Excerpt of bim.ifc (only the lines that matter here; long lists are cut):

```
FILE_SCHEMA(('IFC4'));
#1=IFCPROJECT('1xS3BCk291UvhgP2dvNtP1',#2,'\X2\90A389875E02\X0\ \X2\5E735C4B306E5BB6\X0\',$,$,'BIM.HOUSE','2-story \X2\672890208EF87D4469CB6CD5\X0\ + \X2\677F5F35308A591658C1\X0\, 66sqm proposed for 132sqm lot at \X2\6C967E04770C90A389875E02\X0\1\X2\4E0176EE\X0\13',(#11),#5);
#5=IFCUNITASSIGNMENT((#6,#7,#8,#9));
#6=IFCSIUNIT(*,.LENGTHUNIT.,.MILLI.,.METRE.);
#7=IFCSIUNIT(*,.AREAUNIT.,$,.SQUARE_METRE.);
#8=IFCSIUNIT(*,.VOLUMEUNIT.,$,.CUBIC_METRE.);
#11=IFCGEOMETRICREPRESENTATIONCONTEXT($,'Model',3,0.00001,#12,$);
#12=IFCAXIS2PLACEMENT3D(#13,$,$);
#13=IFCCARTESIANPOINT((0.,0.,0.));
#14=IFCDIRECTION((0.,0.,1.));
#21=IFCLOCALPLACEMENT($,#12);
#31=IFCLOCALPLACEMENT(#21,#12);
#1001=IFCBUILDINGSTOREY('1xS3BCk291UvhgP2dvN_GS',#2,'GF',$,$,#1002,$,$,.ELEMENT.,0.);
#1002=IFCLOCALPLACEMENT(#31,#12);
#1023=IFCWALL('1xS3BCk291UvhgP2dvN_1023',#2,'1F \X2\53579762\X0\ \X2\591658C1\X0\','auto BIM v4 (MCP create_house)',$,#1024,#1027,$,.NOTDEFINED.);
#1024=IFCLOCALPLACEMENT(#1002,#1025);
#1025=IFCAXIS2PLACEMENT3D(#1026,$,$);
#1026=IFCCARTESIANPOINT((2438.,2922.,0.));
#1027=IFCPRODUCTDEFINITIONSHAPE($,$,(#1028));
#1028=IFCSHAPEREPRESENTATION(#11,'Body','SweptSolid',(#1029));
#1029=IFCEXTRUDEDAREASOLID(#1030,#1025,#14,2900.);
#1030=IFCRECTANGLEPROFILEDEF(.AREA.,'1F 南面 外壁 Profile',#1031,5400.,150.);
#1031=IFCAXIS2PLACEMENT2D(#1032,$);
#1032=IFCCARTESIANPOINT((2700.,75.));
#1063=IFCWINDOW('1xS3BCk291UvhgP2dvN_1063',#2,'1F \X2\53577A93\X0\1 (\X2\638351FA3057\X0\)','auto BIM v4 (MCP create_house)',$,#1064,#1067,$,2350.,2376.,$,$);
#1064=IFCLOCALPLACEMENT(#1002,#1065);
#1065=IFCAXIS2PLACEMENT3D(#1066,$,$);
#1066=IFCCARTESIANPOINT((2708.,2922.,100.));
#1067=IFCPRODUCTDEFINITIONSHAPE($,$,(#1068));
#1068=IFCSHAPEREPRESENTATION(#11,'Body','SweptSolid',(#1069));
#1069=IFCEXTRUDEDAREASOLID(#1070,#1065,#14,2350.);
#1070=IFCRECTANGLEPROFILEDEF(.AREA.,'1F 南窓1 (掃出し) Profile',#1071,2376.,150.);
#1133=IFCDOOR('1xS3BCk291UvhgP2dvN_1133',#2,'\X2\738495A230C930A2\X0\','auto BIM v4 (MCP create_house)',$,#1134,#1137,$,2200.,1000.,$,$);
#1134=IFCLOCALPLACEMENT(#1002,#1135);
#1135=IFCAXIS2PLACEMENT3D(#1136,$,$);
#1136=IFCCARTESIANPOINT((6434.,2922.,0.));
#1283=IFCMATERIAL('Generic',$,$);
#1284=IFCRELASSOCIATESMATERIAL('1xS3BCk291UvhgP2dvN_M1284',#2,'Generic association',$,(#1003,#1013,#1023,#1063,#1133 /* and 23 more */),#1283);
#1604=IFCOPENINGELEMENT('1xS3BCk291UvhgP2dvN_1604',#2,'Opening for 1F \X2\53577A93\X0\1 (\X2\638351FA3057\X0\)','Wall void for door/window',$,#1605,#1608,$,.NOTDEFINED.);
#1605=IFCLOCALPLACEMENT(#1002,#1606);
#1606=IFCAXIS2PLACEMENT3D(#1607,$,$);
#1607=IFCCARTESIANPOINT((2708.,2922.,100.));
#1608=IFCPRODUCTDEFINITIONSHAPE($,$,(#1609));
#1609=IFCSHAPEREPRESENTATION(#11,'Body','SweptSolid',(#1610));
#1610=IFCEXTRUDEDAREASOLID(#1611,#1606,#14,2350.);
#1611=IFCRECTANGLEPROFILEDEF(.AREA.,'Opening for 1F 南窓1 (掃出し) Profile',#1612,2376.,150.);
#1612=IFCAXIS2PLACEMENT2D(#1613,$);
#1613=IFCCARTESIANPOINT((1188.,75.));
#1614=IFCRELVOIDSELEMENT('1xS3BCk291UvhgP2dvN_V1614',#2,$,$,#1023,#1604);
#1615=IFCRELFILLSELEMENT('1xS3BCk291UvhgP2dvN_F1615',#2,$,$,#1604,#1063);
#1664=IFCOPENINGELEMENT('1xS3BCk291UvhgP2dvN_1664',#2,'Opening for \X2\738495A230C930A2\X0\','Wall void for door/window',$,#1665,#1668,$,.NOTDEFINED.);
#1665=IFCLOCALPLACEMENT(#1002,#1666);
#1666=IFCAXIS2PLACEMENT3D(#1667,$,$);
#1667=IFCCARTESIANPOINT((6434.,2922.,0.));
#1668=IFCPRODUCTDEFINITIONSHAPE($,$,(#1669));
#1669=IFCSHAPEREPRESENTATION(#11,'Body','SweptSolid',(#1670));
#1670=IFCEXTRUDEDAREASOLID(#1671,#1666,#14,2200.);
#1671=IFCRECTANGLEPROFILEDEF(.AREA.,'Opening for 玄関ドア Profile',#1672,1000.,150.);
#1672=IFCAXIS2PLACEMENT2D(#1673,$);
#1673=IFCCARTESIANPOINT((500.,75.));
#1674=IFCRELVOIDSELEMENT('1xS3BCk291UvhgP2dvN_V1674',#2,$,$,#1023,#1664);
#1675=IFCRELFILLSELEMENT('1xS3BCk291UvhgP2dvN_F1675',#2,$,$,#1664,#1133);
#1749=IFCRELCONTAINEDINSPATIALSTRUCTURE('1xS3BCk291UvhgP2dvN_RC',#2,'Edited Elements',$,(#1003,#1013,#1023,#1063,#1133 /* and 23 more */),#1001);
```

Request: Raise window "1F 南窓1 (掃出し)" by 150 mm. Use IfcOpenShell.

```python
import numpy as np
import ifcopenshell
import ifcopenshell.api.geometry
import ifcopenshell.util.placement
import ifcopenshell.util.unit

model = ifcopenshell.open("bim.ifc")
unit_scale = ifcopenshell.util.unit.calculate_unit_scale(model)

window = model.by_guid("1xS3BCk291UvhgP2dvN_1063")
opening = window.FillsVoids[0].RelatingOpeningElement
dz = 0.15 / unit_scale

shift = np.array([0.0, 0.0, dz])
# The window is not placed relative to its opening, so move both.
for product in (opening, window):
    matrix = ifcopenshell.util.placement.get_local_placement(product.ObjectPlacement)
    matrix[:3, 3] += shift
    ifcopenshell.api.geometry.edit_object_placement(model, product=product, matrix=matrix, is_si=False)

print(f"moved by {dz * unit_scale:+.3f} m")

model.write("bim_updated.ifc")
```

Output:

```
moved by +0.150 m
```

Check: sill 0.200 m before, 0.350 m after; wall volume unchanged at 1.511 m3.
